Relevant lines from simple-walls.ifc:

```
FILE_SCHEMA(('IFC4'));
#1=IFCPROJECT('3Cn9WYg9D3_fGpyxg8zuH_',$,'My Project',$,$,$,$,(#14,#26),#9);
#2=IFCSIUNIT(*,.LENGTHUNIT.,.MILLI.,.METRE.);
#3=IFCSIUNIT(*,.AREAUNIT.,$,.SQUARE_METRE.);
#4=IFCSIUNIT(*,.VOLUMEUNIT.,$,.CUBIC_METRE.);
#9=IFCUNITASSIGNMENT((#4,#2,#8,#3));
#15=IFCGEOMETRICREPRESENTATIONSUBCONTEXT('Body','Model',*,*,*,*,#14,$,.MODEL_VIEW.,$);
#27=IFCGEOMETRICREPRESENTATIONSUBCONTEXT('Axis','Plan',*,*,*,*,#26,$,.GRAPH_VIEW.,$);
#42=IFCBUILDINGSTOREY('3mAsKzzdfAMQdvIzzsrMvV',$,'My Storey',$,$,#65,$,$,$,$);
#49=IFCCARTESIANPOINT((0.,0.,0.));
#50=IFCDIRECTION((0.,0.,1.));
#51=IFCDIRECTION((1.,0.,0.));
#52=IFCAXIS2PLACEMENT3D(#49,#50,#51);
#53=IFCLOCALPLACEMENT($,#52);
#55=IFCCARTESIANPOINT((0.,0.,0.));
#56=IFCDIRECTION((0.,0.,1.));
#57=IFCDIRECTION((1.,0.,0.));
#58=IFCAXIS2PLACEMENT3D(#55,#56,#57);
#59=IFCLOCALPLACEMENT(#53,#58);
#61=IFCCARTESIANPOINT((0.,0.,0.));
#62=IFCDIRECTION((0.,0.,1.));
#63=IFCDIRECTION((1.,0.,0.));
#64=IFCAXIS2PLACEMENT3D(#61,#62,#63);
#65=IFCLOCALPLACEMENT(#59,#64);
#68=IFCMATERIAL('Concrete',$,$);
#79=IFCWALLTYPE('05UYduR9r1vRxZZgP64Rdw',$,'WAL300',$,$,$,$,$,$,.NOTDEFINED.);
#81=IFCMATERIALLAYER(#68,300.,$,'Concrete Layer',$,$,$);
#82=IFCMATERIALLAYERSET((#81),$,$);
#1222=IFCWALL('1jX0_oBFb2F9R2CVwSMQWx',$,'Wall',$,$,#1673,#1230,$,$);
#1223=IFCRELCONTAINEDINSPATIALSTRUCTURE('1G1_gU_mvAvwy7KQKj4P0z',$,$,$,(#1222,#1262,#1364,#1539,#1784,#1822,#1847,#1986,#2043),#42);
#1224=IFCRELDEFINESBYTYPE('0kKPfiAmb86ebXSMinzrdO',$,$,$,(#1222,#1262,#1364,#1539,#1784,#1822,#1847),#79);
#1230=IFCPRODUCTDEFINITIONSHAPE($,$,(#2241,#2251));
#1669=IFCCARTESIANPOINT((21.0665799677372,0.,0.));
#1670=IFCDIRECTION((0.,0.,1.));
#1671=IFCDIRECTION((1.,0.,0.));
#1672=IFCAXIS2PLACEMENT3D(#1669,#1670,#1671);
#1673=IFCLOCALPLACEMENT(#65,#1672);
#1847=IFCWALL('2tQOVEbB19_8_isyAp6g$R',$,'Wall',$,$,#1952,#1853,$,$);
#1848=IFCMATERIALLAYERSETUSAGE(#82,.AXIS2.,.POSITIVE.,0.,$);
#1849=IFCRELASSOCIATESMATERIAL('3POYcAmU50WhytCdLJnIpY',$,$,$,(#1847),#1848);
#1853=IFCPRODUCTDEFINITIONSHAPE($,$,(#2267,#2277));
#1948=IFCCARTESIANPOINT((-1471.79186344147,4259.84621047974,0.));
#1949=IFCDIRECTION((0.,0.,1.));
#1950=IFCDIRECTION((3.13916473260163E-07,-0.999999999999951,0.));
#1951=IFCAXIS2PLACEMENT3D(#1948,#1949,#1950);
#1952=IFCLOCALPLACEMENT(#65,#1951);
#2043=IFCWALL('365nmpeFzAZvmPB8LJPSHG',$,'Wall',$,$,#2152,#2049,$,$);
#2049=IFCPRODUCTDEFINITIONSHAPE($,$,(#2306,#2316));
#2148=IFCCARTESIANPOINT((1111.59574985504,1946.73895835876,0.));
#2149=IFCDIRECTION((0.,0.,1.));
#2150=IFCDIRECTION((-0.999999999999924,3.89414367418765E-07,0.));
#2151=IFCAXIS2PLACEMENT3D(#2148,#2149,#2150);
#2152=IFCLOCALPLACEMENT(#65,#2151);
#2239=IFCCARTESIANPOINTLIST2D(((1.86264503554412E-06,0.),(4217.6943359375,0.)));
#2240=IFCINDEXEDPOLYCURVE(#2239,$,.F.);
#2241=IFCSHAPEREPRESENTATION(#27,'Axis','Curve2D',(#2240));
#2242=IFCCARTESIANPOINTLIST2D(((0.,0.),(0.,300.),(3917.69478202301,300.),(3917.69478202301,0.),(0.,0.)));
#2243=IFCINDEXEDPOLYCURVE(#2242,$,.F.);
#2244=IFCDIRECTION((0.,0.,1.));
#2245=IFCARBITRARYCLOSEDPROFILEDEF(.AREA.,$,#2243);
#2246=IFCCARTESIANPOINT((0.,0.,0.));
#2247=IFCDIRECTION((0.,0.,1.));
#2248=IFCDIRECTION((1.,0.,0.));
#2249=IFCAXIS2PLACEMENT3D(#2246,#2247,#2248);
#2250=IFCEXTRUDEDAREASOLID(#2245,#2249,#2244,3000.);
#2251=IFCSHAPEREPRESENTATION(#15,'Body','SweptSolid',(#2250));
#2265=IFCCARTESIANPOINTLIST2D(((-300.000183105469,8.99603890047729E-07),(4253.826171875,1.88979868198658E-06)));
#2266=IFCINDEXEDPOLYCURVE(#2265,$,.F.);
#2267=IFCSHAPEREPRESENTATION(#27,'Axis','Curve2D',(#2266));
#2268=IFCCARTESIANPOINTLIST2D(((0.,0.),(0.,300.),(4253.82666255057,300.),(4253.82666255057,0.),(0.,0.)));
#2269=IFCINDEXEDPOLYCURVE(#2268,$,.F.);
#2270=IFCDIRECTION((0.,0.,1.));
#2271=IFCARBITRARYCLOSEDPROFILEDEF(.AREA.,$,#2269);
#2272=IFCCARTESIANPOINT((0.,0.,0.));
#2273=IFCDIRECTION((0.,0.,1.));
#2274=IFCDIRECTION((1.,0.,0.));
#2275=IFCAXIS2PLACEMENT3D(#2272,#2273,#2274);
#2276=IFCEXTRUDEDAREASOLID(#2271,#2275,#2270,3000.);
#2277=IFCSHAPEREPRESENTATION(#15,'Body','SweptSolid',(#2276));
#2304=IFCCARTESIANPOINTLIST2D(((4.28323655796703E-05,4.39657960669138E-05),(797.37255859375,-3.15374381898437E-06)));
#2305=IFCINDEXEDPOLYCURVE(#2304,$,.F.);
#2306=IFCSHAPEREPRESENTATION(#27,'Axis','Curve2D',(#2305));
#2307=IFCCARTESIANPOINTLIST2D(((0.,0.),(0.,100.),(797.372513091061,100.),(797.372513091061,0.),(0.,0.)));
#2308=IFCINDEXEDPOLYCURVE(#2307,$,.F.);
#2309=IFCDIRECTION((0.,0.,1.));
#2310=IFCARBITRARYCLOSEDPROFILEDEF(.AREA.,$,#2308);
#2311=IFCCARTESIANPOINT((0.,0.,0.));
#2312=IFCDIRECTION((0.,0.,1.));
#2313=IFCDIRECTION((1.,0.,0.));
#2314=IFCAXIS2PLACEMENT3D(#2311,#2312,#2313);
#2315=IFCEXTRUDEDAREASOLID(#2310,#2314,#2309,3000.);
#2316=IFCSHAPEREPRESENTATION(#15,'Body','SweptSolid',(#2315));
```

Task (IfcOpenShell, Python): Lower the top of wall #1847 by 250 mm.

```python
import ifcopenshell
import ifcopenshell.geom
import ifcopenshell.util.representation
import ifcopenshell.util.shape
import ifcopenshell.util.unit

model = ifcopenshell.open("simple-walls.ifc")
unit_scale = ifcopenshell.util.unit.calculate_unit_scale(model)
settings = ifcopenshell.geom.settings()


def volume(element):
    """Net volume in cubic metres, openings subtracted."""
    shape = ifcopenshell.geom.create_shape(settings, element)
    return ifcopenshell.util.shape.get_volume(shape.geometry)


wall = model.by_id(1847)
before = volume(wall)

body = ifcopenshell.util.representation.get_representation(wall, "Model", "Body")
solid = body.Items[0]
old_height = solid.Depth
solid.Depth -= 0.25 / unit_scale
after = volume(wall)

print(f"height {old_height:g} -> {solid.Depth:g}, volume {before:.3f} -> {after:.3f} m3")

model.write("simple-walls_edited.ifc")
```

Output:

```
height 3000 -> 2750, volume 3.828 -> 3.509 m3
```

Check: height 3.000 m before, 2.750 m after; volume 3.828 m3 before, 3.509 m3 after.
